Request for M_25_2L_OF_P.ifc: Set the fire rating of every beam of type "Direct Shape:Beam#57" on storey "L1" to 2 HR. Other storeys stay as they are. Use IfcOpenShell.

First a look at what the model holds.

```python
import ifcopenshell
import ifcopenshell.util.element

model = ifcopenshell.open("M_25_2L_OF_P.ifc")
print(model.schema)
storey = next(s for s in model.by_type("IfcBuildingStorey") if s.Name == "L1")
beams = [e for e in ifcopenshell.util.element.get_decomposition(storey) if e.is_a("IfcBeam")]
seen = {}
for e in beams:
    element_type = ifcopenshell.util.element.get_type(e)
    key = (element_type.Name if element_type != e and element_type else None, ifcopenshell.util.element.get_pset(e, "Pset_BeamCommon", "FireRating"))
    seen[key] = seen.get(key, 0) + 1
for (name, value), count in sorted(seen.items(), key=str):
    print(count, "x", name, "|", value)
```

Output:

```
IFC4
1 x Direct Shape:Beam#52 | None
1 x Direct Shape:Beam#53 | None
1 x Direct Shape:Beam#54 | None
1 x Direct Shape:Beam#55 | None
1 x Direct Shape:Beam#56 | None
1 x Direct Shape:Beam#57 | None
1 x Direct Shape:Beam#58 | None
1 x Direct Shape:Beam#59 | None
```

```python
import ifcopenshell
import ifcopenshell.api.pset
import ifcopenshell.util.element

model = ifcopenshell.open("M_25_2L_OF_P.ifc")

storey = next(s for s in model.by_type("IfcBuildingStorey") if s.Name == "L1")
beams = [e for e in ifcopenshell.util.element.get_decomposition(storey) if e.is_a("IfcBeam")]

count = 0
for e in beams:
    element_type = ifcopenshell.util.element.get_type(e)
    if element_type in (None, e) or element_type.Name != "Direct Shape:Beam#57":
        continue
    # add_pset returns the element's existing set when there is one.
    pset = ifcopenshell.api.pset.add_pset(model, product=e, name="Pset_BeamCommon")
    ifcopenshell.api.pset.edit_pset(model, pset=pset, properties={"FireRating": "2 HR"})
    count += 1

print(count, "beams updated")

model.write("M_25_2L_OF_P_edited.ifc")
```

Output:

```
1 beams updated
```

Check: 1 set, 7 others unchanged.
